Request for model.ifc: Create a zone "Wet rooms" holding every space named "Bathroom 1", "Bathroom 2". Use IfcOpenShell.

First a look at what the model holds.

```python
import ifcopenshell

model = ifcopenshell.open("model.ifc")
print(model.schema)
seen = {}
for space in model.by_type("IfcSpace"):
    seen[space.LongName] = seen.get(space.LongName, 0) + 1
for name, count in sorted(seen.items(), key=str):
    print(count, "x", name)
print("zones:", [z.Name for z in model.by_type("IfcZone")][:20])
```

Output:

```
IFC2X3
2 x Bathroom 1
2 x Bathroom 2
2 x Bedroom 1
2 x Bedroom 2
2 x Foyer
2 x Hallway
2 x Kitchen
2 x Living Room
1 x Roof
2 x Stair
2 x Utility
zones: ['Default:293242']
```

```python
import ifcopenshell
import ifcopenshell.api.group
import ifcopenshell.api.root

model = ifcopenshell.open("model.ifc")

names = {"Bathroom 1", "Bathroom 2"}
spaces = [s for s in model.by_type("IfcSpace") if s.LongName in names]

zone = ifcopenshell.api.root.create_entity(model, ifc_class="IfcZone", name="Wet rooms")
ifcopenshell.api.group.assign_group(model, products=spaces, group=zone)
print(len(spaces), "spaces in", zone.Name)

model.write("model-out.ifc")
```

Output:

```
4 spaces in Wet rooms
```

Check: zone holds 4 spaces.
